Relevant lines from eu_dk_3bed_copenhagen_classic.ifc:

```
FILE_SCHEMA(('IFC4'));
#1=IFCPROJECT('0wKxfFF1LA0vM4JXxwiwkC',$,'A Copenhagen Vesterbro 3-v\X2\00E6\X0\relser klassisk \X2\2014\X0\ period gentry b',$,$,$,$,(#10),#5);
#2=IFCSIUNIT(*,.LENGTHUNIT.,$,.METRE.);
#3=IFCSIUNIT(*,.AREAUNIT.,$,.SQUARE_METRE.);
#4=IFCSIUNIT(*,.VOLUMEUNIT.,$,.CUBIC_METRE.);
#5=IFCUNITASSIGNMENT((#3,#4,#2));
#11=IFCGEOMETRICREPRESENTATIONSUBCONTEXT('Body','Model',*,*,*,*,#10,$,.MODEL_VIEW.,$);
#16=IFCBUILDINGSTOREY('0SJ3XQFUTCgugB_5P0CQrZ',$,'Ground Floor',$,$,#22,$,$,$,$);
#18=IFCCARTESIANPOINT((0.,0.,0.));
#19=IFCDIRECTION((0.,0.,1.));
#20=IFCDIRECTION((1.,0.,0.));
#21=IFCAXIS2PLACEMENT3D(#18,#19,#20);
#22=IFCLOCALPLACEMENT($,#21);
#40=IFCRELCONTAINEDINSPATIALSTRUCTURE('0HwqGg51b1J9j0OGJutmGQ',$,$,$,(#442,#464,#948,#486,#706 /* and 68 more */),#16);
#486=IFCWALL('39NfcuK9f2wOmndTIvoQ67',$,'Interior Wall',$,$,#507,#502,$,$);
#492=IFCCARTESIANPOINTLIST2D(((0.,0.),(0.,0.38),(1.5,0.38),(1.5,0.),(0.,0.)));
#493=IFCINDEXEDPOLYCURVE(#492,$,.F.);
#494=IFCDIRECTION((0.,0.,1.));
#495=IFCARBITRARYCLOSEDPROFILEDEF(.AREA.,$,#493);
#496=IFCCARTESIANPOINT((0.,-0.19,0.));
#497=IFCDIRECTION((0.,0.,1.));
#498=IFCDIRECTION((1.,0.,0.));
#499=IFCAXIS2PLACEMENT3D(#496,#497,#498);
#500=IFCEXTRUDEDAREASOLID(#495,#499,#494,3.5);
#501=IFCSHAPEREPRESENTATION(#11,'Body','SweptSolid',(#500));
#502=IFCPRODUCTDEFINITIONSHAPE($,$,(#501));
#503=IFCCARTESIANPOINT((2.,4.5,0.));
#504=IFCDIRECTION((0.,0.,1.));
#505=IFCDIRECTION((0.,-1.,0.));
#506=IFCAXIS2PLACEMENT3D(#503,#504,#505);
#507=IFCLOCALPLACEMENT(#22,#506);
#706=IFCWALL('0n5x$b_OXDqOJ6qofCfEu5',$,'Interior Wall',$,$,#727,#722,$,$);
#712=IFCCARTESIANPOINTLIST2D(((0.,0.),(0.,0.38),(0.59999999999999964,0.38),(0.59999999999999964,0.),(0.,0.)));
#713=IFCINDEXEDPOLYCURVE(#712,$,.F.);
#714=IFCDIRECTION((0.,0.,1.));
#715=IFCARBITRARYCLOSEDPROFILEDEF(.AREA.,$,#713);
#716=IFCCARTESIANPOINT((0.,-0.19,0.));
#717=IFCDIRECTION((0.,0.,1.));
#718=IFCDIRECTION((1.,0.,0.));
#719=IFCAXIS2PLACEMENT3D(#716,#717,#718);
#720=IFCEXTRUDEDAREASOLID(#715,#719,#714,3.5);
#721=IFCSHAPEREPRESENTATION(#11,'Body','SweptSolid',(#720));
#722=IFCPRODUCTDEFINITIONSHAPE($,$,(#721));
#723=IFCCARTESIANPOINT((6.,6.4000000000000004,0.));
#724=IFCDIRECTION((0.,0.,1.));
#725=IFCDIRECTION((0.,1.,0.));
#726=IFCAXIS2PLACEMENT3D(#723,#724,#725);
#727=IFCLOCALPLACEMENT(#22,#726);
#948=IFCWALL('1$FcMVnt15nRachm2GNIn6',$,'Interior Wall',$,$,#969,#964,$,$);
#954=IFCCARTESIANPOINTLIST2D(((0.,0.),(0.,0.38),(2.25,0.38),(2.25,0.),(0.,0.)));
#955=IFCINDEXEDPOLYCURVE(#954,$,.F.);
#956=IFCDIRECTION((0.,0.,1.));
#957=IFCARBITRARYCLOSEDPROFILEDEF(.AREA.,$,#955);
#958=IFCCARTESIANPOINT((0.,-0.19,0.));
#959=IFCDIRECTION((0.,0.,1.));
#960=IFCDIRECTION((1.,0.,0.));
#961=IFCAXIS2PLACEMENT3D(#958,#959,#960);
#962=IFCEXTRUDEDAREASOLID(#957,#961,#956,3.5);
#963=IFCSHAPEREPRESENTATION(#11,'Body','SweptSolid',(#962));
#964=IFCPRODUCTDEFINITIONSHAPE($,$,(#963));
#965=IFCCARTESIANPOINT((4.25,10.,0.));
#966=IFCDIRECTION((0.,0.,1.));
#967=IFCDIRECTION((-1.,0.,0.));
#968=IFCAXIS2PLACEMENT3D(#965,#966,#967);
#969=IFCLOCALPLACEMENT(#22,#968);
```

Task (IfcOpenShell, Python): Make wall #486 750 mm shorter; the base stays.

```python
import ifcopenshell
import ifcopenshell.geom
import ifcopenshell.util.representation
import ifcopenshell.util.shape
import ifcopenshell.util.unit

model = ifcopenshell.open("eu_dk_3bed_copenhagen_classic.ifc")
unit_scale = ifcopenshell.util.unit.calculate_unit_scale(model)
settings = ifcopenshell.geom.settings()


def volume(element):
    """Net volume in cubic metres, openings subtracted."""
    shape = ifcopenshell.geom.create_shape(settings, element)
    return ifcopenshell.util.shape.get_volume(shape.geometry)


wall = model.by_guid("39NfcuK9f2wOmndTIvoQ67")
before = volume(wall)

body = ifcopenshell.util.representation.get_representation(wall, "Model", "Body")
solid = body.Items[0]
old_height = solid.Depth
solid.Depth -= 0.75 / unit_scale
after = volume(wall)

print(f"height {old_height:g} -> {solid.Depth:g}, volume {before:.3f} -> {after:.3f} m3")

model.write("eu_dk_3bed_copenhagen_classic_updated.ifc")
```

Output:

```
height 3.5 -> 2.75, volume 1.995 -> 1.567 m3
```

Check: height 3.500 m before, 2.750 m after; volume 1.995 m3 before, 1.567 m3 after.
